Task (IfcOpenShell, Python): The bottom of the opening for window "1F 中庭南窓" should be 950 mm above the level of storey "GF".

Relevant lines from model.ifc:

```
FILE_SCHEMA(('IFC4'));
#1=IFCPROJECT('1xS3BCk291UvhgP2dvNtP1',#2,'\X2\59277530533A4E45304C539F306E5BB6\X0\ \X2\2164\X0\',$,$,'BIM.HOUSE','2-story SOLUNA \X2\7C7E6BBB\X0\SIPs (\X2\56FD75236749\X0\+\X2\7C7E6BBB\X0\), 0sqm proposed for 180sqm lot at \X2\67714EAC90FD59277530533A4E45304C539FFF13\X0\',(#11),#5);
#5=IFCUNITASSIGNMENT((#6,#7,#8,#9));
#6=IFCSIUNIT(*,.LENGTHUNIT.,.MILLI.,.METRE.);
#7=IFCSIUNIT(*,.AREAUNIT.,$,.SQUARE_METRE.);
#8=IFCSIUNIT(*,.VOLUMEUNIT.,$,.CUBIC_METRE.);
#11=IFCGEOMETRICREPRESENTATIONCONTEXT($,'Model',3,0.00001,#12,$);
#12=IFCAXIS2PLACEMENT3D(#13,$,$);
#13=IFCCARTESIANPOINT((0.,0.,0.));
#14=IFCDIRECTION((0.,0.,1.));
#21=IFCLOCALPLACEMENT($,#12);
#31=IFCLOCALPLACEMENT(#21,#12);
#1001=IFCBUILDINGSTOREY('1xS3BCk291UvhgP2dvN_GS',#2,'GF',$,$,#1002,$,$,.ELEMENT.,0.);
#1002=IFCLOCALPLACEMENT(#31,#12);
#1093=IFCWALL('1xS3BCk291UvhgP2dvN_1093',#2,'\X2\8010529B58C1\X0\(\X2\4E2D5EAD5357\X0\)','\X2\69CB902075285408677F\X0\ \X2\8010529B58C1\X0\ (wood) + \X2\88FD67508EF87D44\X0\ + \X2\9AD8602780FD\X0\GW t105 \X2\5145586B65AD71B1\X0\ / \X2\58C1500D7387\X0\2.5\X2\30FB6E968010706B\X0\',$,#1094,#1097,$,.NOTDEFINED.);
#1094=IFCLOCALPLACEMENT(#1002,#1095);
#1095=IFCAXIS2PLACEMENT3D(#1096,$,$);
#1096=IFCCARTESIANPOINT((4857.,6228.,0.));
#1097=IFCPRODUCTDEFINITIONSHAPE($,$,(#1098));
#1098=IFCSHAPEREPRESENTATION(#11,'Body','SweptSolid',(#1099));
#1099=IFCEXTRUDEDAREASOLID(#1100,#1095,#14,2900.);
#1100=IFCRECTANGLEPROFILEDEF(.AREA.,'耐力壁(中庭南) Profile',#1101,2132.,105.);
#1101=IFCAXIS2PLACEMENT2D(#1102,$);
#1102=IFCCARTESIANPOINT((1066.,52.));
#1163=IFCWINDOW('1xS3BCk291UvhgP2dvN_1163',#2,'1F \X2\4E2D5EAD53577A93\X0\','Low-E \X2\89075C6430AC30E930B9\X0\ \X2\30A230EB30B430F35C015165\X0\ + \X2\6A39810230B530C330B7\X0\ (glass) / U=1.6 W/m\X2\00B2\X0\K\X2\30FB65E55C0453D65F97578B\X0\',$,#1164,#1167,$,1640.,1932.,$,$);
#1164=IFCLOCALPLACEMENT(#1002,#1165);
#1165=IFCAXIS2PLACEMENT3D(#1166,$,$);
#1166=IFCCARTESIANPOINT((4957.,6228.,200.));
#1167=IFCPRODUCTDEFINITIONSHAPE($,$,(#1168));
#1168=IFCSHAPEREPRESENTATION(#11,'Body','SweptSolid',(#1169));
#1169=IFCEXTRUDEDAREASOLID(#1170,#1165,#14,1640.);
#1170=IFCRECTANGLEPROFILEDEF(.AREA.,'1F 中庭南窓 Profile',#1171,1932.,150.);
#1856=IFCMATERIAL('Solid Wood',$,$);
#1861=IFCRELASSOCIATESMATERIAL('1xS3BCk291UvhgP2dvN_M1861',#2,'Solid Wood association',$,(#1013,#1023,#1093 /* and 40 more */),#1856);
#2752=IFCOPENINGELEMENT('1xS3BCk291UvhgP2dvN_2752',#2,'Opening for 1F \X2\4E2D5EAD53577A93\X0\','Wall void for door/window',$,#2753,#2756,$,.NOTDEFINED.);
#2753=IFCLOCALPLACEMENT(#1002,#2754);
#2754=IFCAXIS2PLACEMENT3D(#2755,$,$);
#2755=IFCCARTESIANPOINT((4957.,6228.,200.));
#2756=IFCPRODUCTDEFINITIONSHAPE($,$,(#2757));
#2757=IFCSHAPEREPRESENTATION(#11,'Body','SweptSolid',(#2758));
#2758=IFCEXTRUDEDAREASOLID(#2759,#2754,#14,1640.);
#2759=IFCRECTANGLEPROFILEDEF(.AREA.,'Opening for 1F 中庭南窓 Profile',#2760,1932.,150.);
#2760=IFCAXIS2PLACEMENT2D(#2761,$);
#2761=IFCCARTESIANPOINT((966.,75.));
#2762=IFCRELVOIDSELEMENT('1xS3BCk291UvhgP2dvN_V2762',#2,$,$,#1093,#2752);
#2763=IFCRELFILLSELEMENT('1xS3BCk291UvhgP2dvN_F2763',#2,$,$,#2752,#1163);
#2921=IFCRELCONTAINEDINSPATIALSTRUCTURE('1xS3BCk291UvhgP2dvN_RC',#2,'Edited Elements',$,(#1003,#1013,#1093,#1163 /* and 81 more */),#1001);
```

```python
import numpy as np
import ifcopenshell
import ifcopenshell.api.geometry
import ifcopenshell.geom
import ifcopenshell.util.element
import ifcopenshell.util.placement
import ifcopenshell.util.shape
import ifcopenshell.util.unit

model = ifcopenshell.open("model.ifc")
unit_scale = ifcopenshell.util.unit.calculate_unit_scale(model)

window = model.by_id(1163)
opening = window.FillsVoids[0].RelatingOpeningElement
storey = ifcopenshell.util.element.get_container(window, ifc_class="IfcBuildingStorey")
level = ifcopenshell.util.placement.get_local_placement(storey.ObjectPlacement)[2, 3]

# The opening's origin need not be at the sill, so measure its lowest point.
shape = ifcopenshell.geom.create_shape(ifcopenshell.geom.settings(), opening)
bottom = ifcopenshell.util.shape.get_shape_bottom_elevation(shape, shape.geometry) / unit_scale
dz = level + 0.95 / unit_scale - bottom

shift = np.array([0.0, 0.0, dz])
# The window is not placed relative to its opening, so move both.
for product in (opening, window):
    matrix = ifcopenshell.util.placement.get_local_placement(product.ObjectPlacement)
    matrix[:3, 3] += shift
    ifcopenshell.api.geometry.edit_object_placement(model, product=product, matrix=matrix, is_si=False)

print(f"moved by {dz * unit_scale:+.3f} m")

model.write("model_v2.ifc")
```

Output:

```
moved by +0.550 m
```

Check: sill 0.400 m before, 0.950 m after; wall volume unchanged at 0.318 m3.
